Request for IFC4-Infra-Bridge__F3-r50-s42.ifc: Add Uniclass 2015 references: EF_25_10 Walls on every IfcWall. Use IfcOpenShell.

First a look at what the model holds.

```python
import ifcopenshell

model = ifcopenshell.open("IFC4-Infra-Bridge__F3-r50-s42.ifc")
print(model.schema)
print("classifications:", [c.Name for c in model.by_type("IfcClassification")])
for ifc_class in ("IfcDoor", "IfcRoof", "IfcStair", "IfcWall", "IfcWindow"):
    print(ifc_class, len(model.by_type(ifc_class)))
```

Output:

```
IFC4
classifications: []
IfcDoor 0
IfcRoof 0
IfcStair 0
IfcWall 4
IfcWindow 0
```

```python
import ifcopenshell
import ifcopenshell.api.classification

model = ifcopenshell.open("IFC4-Infra-Bridge__F3-r50-s42.ifc")

system = ifcopenshell.api.classification.add_classification(model, classification="Uniclass 2015")

codes = {
    "IfcWall": ("EF_25_10", "Walls"),
}
for ifc_class, (code, name) in codes.items():
    products = model.by_type(ifc_class)
    ifcopenshell.api.classification.add_reference(
        model, products=products, classification=system, identification=code, name=name
    )
    print(code, len(products))

model.write("IFC4-Infra-Bridge__F3-r50-s42_v2.ifc")
```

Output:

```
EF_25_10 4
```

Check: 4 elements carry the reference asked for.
